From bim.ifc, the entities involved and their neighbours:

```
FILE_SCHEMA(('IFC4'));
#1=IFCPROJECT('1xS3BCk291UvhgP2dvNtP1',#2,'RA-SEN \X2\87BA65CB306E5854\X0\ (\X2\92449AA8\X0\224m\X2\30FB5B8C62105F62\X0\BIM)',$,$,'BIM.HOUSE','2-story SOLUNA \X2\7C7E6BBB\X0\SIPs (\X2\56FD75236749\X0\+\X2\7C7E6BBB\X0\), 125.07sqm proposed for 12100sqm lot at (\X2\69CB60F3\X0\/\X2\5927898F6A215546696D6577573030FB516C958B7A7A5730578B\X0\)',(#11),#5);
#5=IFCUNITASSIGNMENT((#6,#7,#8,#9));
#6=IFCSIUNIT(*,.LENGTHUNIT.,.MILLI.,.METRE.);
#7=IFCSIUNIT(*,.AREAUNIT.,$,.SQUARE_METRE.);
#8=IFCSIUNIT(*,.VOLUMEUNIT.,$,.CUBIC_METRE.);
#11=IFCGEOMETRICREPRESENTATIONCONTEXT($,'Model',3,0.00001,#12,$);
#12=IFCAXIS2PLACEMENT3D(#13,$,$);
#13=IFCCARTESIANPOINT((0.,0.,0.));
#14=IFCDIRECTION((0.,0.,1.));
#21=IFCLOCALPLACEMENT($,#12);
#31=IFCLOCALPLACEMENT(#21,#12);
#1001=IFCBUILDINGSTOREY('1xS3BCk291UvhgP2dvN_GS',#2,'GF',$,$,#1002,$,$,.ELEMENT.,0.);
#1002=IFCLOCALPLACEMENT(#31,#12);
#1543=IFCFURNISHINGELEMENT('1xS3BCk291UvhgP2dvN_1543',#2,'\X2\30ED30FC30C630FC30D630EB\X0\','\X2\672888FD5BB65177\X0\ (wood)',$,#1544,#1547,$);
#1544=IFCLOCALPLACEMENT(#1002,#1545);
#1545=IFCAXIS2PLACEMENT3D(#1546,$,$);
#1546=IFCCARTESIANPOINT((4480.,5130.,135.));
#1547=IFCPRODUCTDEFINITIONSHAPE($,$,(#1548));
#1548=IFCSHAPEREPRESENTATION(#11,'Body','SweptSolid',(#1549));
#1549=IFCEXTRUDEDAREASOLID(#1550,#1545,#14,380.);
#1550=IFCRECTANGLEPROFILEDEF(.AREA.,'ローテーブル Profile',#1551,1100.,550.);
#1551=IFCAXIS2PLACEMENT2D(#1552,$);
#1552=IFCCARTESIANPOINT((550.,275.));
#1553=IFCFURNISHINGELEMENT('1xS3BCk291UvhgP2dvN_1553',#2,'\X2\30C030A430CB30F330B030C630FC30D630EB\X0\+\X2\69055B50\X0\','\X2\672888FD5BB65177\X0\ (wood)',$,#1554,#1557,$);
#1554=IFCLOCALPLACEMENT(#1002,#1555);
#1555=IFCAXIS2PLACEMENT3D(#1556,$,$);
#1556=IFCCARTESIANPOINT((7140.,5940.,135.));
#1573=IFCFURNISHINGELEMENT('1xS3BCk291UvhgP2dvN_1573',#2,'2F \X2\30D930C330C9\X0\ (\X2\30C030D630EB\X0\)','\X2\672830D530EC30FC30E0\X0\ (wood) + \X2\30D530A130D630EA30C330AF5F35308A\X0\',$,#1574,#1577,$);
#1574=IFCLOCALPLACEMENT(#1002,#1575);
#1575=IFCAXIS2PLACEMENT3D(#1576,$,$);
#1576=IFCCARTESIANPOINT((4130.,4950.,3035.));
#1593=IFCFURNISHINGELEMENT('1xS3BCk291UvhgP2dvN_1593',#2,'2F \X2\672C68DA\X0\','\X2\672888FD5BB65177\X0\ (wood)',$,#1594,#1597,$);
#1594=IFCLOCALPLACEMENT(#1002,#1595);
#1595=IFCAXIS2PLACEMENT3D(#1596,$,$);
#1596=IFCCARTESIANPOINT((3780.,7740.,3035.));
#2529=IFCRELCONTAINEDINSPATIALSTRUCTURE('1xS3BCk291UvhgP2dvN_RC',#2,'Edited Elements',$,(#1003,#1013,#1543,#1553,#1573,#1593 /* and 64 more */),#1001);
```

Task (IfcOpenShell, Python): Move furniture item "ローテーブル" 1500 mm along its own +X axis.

```python
import ifcopenshell
import ifcopenshell.api.geometry
import ifcopenshell.util.placement
import ifcopenshell.util.unit

model = ifcopenshell.open("bim.ifc")
unit_scale = ifcopenshell.util.unit.calculate_unit_scale(model)

item = model.by_guid("1xS3BCk291UvhgP2dvN_1543")
matrix = ifcopenshell.util.placement.get_local_placement(item.ObjectPlacement)
matrix[:3, 3] += matrix[:3, 0] * 1.5 / unit_scale
ifcopenshell.api.geometry.edit_object_placement(model, product=item, matrix=matrix, is_si=False)

print(ifcopenshell.util.placement.get_local_placement(item.ObjectPlacement).round(3) + 0.0)

model.write("bim_rev.ifc")
```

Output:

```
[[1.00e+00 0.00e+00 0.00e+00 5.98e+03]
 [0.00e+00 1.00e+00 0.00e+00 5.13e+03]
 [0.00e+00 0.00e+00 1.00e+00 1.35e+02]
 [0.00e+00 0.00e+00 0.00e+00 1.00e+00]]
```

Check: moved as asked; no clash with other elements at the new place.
